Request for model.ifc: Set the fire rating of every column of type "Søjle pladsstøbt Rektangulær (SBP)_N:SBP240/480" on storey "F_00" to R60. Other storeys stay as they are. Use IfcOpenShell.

First a look at what the model holds.

```python
import ifcopenshell
import ifcopenshell.util.element

model = ifcopenshell.open("model.ifc")
print(model.schema)
storey = next(s for s in model.by_type("IfcBuildingStorey") if s.Name == "F_00")
columns = [e for e in ifcopenshell.util.element.get_decomposition(storey) if e.is_a("IfcColumn")]
seen = {}
for e in columns:
    element_type = ifcopenshell.util.element.get_type(e)
    key = (element_type.Name if element_type != e and element_type else None, ifcopenshell.util.element.get_pset(e, "Pset_ColumnCommon", "FireRating"))
    seen[key] = seen.get(key, 0) + 1
for (name, value), count in sorted(seen.items(), key=str):
    print(count, "x", name, "|", value)
```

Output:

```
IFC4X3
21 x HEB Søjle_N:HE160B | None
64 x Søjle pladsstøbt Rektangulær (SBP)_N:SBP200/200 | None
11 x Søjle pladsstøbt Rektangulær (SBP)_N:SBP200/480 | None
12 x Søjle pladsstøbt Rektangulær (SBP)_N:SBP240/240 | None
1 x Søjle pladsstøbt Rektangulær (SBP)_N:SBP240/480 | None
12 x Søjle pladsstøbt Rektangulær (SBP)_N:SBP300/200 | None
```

```python
import ifcopenshell
import ifcopenshell.api.pset
import ifcopenshell.util.element

model = ifcopenshell.open("model.ifc")

storey = next(s for s in model.by_type("IfcBuildingStorey") if s.Name == "F_00")
columns = [e for e in ifcopenshell.util.element.get_decomposition(storey) if e.is_a("IfcColumn")]

count = 0
for e in columns:
    element_type = ifcopenshell.util.element.get_type(e)
    if element_type in (None, e) or element_type.Name != "Søjle pladsstøbt Rektangulær (SBP)_N:SBP240/480":
        continue
    # add_pset returns the element's existing set when there is one.
    pset = ifcopenshell.api.pset.add_pset(model, product=e, name="Pset_ColumnCommon")
    ifcopenshell.api.pset.edit_pset(model, pset=pset, properties={"FireRating": "R60"})
    count += 1

print(count, "columns updated")

model.write("model_updated.ifc")
```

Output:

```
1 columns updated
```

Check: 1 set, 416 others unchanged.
